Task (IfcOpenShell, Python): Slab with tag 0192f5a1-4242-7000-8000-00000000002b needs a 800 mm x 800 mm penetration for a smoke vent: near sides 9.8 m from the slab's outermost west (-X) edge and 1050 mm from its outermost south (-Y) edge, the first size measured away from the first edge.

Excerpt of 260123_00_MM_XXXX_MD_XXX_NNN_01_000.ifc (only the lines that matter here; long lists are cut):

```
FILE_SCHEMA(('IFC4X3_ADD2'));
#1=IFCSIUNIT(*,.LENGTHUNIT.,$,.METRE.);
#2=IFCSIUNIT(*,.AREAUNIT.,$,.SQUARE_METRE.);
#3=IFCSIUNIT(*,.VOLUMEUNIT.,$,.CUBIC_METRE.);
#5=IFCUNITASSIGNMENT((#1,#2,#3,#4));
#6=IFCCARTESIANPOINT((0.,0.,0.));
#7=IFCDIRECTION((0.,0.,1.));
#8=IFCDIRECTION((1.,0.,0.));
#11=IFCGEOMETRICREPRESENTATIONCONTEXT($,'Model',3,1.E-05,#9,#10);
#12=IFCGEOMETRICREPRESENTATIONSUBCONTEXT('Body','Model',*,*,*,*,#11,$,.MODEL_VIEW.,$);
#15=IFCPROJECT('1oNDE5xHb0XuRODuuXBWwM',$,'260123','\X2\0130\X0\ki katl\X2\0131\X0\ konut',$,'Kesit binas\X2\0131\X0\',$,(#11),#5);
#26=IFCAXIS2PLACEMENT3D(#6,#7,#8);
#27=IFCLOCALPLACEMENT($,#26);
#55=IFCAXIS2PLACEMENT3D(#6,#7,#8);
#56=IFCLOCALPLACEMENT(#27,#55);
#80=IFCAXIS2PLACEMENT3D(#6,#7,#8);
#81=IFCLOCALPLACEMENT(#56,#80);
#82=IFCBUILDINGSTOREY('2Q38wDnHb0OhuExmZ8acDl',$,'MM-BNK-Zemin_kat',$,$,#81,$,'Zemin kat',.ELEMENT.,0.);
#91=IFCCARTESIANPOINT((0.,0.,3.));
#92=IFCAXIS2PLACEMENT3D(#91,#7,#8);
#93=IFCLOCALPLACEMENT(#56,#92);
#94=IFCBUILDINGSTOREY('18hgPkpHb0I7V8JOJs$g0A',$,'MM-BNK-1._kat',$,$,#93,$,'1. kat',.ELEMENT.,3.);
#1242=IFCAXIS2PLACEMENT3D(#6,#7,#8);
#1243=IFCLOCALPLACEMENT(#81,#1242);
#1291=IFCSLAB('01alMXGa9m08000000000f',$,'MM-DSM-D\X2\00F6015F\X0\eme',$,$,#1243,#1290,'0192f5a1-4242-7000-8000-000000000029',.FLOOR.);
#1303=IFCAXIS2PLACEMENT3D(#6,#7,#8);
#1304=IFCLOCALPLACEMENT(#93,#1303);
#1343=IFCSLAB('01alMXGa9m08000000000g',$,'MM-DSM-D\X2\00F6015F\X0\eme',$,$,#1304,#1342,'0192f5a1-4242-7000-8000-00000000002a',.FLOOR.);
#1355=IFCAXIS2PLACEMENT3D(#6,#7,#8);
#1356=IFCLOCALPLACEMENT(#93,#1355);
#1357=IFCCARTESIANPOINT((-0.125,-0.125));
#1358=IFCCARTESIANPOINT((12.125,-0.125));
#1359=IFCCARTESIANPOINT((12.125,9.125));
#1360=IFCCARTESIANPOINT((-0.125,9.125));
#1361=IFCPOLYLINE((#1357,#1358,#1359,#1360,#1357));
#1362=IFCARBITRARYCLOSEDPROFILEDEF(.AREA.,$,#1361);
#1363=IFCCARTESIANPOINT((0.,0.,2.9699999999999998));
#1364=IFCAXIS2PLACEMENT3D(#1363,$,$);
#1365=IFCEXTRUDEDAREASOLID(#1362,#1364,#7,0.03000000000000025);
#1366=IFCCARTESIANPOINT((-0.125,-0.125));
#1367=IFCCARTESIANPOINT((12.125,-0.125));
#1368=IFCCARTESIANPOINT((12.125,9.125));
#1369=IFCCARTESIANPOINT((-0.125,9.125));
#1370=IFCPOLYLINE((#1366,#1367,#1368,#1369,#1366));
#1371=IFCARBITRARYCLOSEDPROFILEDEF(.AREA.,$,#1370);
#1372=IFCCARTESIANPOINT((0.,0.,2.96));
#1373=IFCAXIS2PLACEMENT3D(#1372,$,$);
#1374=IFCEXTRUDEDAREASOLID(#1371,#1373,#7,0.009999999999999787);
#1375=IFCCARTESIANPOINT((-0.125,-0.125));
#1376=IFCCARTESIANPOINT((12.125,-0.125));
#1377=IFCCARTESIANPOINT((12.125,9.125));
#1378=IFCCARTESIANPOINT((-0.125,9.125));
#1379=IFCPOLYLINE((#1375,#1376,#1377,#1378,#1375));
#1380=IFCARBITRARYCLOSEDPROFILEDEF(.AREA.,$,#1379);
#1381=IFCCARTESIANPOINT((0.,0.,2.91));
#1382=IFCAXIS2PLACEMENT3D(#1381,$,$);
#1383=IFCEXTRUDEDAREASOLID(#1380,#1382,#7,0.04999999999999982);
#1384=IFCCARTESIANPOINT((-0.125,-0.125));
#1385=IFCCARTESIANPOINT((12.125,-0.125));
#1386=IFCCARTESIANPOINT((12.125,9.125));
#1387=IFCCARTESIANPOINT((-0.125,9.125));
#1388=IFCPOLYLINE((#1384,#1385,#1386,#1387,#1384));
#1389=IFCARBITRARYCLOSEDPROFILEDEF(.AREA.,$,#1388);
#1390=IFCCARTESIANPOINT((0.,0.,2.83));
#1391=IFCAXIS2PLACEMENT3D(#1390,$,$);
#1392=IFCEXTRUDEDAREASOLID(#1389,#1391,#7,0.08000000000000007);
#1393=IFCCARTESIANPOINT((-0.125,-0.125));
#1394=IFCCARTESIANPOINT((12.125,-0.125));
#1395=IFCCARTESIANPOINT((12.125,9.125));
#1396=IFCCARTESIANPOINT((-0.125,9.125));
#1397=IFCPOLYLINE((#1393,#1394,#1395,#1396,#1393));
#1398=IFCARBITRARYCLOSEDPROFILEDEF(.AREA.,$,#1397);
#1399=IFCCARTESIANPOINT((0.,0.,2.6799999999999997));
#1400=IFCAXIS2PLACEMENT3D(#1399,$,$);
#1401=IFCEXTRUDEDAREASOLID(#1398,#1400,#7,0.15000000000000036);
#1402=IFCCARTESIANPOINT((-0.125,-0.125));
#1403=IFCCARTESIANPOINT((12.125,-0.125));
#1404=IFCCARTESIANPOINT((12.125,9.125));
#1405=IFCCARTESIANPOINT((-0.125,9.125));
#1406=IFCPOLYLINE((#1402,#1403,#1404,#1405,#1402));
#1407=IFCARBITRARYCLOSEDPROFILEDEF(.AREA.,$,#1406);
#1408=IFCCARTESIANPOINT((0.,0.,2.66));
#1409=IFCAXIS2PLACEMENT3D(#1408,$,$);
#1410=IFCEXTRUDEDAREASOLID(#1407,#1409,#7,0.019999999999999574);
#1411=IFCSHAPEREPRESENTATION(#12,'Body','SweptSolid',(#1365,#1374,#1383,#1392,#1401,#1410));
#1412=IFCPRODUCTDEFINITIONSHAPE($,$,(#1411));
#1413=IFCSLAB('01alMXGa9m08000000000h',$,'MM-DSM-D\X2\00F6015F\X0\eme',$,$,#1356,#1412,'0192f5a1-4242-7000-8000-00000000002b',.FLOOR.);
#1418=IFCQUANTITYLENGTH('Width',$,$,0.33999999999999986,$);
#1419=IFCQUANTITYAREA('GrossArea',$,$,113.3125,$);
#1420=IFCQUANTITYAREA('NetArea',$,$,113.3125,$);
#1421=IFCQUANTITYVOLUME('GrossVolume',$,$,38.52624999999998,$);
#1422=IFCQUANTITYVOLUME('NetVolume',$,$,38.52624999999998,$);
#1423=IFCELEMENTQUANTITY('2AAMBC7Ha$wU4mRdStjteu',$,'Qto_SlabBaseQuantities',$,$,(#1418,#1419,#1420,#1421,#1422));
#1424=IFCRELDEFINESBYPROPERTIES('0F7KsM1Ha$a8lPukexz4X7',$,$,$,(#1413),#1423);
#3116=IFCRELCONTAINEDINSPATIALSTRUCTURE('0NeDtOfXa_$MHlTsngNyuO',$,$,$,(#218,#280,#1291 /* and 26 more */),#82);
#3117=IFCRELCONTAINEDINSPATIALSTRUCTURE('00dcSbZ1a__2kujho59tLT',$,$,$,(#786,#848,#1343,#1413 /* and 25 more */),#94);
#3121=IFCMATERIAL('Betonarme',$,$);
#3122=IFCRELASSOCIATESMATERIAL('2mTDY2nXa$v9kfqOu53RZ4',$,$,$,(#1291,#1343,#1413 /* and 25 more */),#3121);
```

```python
import numpy as np
import ifcopenshell
import ifcopenshell.api.feature
import ifcopenshell.api.geometry
import ifcopenshell.api.pset
import ifcopenshell.api.root
import ifcopenshell.geom
import ifcopenshell.util.element
import ifcopenshell.util.placement
import ifcopenshell.util.representation
import ifcopenshell.util.shape
import ifcopenshell.util.unit

model = ifcopenshell.open("260123_00_MM_XXXX_MD_XXX_NNN_01_000.ifc")
unit_scale = ifcopenshell.util.unit.calculate_unit_scale(model)
area_scale = ifcopenshell.util.unit.calculate_unit_scale(model, "AREAUNIT")
volume_scale = ifcopenshell.util.unit.calculate_unit_scale(model, "VOLUMEUNIT")
settings = ifcopenshell.geom.settings()


def volume(element):
    """Net volume in cubic metres, openings subtracted."""
    shape = ifcopenshell.geom.create_shape(settings, element)
    return ifcopenshell.util.shape.get_volume(shape.geometry)


slab = model.by_guid("01alMXGa9m08000000000h")
before = volume(slab)

# Extent in the slab's own axes, in metres. The edges named are its -X and -Y sides.
slab_shape = ifcopenshell.geom.create_shape(settings, slab)
vertices = ifcopenshell.util.shape.get_vertices(slab_shape.geometry)
x_min, y_min, bottom = vertices.min(axis=0)
top = vertices[:, 2].max()

opening = ifcopenshell.api.root.create_entity(model, ifc_class="IfcOpeningElement", name="Smoke vent opening", predefined_type="OPENING")
context = ifcopenshell.util.representation.get_context(model, "Model", "Body", "MODEL_VIEW")
width, depth = 0.8, 0.8
outline = [(0.0, 0.0), (width, 0.0), (width, depth), (0.0, depth), (0.0, 0.0)]
# Overshoot both faces by 50 mm so the cut is clean.
shape = ifcopenshell.api.geometry.add_slab_representation(
    model, context=context, depth=top - bottom + 0.1, polyline=outline
)
ifcopenshell.api.geometry.assign_representation(model, product=opening, representation=shape)

matrix = ifcopenshell.util.placement.get_local_placement(slab.ObjectPlacement)
matrix[:, 3] = matrix @ np.append(np.array([x_min + 9.8, y_min + 1.05, bottom - 0.05]) / unit_scale, 1.0)
ifcopenshell.api.geometry.edit_object_placement(model, product=opening, matrix=matrix, is_si=False)
ifcopenshell.api.feature.add_feature(model, feature=opening, element=slab)

after = volume(slab)

# Update the slab's stored quantities.
qto = model.by_id(ifcopenshell.util.element.get_pset(slab, "Qto_SlabBaseQuantities", should_inherit=False)["id"])
ifcopenshell.api.pset.edit_qto(model, qto=qto, properties={
    "NetArea": after / (top - bottom) / area_scale,
    "NetVolume": after / volume_scale,
})

print(f"slab volume {before:.3f} -> {after:.3f} m3")

model.write("260123_00_MM_XXXX_MD_XXX_NNN_01_000-out.ifc")
```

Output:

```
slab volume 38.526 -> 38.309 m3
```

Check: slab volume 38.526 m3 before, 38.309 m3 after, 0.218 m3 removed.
